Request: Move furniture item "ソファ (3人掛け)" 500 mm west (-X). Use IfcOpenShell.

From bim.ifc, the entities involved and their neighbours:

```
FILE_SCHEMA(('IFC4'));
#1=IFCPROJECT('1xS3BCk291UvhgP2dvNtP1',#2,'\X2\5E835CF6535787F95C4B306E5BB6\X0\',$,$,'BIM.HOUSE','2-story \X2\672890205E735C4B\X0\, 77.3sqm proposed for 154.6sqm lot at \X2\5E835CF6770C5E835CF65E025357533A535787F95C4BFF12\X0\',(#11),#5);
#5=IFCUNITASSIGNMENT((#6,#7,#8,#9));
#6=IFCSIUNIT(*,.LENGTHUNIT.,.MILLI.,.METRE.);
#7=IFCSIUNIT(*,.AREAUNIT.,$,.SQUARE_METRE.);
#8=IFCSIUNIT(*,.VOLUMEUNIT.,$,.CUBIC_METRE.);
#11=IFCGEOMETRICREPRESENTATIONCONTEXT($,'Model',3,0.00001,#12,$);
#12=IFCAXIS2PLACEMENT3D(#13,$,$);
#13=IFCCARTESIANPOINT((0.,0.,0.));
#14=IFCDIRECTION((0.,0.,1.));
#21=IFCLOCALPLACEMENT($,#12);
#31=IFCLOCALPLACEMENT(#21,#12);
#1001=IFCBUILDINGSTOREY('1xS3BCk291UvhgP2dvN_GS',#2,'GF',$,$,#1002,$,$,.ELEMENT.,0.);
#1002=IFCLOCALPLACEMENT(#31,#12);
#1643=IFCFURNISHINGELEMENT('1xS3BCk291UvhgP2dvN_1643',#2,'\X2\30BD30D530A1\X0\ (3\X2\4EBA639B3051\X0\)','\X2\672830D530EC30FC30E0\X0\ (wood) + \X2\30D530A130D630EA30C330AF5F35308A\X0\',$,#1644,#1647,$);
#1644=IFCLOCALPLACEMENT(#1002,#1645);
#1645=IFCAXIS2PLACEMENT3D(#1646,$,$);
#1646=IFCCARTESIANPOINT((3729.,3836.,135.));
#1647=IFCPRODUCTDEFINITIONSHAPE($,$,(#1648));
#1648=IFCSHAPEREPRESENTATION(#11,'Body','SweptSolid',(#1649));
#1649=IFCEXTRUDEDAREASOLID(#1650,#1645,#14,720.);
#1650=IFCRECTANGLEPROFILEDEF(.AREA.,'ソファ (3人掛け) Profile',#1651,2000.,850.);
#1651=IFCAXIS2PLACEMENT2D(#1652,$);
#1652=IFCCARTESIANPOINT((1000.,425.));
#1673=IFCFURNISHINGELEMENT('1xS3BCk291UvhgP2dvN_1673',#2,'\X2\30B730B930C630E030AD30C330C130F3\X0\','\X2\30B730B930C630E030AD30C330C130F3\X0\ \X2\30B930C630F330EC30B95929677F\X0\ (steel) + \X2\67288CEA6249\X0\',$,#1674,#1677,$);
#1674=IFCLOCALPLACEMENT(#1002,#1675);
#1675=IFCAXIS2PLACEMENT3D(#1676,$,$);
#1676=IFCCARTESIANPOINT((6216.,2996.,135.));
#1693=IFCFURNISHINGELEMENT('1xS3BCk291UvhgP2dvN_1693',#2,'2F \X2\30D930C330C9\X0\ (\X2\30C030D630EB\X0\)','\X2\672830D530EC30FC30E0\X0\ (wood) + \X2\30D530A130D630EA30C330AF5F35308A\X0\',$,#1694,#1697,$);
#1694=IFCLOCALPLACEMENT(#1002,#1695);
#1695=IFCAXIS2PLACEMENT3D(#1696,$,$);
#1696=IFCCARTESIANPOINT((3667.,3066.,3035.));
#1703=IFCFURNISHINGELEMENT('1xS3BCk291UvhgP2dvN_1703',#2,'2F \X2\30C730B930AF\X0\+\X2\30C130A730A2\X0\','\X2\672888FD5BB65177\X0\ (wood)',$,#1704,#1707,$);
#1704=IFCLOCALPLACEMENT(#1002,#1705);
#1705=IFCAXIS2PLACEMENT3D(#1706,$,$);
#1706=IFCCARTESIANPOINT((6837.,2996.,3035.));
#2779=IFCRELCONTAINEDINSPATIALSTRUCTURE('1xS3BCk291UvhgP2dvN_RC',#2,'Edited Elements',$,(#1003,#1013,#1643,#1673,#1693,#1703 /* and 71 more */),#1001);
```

```python
import ifcopenshell
import ifcopenshell.api.geometry
import ifcopenshell.util.placement

model = ifcopenshell.open("bim.ifc")

item = model.by_id(1643)
matrix = ifcopenshell.util.placement.get_local_placement(item.ObjectPlacement)
matrix[0, 3] -= 500.0
ifcopenshell.api.geometry.edit_object_placement(model, product=item, matrix=matrix, is_si=False)

print(ifcopenshell.util.placement.get_local_placement(item.ObjectPlacement).round(3) + 0.0)

model.write("bim_edited.ifc")
```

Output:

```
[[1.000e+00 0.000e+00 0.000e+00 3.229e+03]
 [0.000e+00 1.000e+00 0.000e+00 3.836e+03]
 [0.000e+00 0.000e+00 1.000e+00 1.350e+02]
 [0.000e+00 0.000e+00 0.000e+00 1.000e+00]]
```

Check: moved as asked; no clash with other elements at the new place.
